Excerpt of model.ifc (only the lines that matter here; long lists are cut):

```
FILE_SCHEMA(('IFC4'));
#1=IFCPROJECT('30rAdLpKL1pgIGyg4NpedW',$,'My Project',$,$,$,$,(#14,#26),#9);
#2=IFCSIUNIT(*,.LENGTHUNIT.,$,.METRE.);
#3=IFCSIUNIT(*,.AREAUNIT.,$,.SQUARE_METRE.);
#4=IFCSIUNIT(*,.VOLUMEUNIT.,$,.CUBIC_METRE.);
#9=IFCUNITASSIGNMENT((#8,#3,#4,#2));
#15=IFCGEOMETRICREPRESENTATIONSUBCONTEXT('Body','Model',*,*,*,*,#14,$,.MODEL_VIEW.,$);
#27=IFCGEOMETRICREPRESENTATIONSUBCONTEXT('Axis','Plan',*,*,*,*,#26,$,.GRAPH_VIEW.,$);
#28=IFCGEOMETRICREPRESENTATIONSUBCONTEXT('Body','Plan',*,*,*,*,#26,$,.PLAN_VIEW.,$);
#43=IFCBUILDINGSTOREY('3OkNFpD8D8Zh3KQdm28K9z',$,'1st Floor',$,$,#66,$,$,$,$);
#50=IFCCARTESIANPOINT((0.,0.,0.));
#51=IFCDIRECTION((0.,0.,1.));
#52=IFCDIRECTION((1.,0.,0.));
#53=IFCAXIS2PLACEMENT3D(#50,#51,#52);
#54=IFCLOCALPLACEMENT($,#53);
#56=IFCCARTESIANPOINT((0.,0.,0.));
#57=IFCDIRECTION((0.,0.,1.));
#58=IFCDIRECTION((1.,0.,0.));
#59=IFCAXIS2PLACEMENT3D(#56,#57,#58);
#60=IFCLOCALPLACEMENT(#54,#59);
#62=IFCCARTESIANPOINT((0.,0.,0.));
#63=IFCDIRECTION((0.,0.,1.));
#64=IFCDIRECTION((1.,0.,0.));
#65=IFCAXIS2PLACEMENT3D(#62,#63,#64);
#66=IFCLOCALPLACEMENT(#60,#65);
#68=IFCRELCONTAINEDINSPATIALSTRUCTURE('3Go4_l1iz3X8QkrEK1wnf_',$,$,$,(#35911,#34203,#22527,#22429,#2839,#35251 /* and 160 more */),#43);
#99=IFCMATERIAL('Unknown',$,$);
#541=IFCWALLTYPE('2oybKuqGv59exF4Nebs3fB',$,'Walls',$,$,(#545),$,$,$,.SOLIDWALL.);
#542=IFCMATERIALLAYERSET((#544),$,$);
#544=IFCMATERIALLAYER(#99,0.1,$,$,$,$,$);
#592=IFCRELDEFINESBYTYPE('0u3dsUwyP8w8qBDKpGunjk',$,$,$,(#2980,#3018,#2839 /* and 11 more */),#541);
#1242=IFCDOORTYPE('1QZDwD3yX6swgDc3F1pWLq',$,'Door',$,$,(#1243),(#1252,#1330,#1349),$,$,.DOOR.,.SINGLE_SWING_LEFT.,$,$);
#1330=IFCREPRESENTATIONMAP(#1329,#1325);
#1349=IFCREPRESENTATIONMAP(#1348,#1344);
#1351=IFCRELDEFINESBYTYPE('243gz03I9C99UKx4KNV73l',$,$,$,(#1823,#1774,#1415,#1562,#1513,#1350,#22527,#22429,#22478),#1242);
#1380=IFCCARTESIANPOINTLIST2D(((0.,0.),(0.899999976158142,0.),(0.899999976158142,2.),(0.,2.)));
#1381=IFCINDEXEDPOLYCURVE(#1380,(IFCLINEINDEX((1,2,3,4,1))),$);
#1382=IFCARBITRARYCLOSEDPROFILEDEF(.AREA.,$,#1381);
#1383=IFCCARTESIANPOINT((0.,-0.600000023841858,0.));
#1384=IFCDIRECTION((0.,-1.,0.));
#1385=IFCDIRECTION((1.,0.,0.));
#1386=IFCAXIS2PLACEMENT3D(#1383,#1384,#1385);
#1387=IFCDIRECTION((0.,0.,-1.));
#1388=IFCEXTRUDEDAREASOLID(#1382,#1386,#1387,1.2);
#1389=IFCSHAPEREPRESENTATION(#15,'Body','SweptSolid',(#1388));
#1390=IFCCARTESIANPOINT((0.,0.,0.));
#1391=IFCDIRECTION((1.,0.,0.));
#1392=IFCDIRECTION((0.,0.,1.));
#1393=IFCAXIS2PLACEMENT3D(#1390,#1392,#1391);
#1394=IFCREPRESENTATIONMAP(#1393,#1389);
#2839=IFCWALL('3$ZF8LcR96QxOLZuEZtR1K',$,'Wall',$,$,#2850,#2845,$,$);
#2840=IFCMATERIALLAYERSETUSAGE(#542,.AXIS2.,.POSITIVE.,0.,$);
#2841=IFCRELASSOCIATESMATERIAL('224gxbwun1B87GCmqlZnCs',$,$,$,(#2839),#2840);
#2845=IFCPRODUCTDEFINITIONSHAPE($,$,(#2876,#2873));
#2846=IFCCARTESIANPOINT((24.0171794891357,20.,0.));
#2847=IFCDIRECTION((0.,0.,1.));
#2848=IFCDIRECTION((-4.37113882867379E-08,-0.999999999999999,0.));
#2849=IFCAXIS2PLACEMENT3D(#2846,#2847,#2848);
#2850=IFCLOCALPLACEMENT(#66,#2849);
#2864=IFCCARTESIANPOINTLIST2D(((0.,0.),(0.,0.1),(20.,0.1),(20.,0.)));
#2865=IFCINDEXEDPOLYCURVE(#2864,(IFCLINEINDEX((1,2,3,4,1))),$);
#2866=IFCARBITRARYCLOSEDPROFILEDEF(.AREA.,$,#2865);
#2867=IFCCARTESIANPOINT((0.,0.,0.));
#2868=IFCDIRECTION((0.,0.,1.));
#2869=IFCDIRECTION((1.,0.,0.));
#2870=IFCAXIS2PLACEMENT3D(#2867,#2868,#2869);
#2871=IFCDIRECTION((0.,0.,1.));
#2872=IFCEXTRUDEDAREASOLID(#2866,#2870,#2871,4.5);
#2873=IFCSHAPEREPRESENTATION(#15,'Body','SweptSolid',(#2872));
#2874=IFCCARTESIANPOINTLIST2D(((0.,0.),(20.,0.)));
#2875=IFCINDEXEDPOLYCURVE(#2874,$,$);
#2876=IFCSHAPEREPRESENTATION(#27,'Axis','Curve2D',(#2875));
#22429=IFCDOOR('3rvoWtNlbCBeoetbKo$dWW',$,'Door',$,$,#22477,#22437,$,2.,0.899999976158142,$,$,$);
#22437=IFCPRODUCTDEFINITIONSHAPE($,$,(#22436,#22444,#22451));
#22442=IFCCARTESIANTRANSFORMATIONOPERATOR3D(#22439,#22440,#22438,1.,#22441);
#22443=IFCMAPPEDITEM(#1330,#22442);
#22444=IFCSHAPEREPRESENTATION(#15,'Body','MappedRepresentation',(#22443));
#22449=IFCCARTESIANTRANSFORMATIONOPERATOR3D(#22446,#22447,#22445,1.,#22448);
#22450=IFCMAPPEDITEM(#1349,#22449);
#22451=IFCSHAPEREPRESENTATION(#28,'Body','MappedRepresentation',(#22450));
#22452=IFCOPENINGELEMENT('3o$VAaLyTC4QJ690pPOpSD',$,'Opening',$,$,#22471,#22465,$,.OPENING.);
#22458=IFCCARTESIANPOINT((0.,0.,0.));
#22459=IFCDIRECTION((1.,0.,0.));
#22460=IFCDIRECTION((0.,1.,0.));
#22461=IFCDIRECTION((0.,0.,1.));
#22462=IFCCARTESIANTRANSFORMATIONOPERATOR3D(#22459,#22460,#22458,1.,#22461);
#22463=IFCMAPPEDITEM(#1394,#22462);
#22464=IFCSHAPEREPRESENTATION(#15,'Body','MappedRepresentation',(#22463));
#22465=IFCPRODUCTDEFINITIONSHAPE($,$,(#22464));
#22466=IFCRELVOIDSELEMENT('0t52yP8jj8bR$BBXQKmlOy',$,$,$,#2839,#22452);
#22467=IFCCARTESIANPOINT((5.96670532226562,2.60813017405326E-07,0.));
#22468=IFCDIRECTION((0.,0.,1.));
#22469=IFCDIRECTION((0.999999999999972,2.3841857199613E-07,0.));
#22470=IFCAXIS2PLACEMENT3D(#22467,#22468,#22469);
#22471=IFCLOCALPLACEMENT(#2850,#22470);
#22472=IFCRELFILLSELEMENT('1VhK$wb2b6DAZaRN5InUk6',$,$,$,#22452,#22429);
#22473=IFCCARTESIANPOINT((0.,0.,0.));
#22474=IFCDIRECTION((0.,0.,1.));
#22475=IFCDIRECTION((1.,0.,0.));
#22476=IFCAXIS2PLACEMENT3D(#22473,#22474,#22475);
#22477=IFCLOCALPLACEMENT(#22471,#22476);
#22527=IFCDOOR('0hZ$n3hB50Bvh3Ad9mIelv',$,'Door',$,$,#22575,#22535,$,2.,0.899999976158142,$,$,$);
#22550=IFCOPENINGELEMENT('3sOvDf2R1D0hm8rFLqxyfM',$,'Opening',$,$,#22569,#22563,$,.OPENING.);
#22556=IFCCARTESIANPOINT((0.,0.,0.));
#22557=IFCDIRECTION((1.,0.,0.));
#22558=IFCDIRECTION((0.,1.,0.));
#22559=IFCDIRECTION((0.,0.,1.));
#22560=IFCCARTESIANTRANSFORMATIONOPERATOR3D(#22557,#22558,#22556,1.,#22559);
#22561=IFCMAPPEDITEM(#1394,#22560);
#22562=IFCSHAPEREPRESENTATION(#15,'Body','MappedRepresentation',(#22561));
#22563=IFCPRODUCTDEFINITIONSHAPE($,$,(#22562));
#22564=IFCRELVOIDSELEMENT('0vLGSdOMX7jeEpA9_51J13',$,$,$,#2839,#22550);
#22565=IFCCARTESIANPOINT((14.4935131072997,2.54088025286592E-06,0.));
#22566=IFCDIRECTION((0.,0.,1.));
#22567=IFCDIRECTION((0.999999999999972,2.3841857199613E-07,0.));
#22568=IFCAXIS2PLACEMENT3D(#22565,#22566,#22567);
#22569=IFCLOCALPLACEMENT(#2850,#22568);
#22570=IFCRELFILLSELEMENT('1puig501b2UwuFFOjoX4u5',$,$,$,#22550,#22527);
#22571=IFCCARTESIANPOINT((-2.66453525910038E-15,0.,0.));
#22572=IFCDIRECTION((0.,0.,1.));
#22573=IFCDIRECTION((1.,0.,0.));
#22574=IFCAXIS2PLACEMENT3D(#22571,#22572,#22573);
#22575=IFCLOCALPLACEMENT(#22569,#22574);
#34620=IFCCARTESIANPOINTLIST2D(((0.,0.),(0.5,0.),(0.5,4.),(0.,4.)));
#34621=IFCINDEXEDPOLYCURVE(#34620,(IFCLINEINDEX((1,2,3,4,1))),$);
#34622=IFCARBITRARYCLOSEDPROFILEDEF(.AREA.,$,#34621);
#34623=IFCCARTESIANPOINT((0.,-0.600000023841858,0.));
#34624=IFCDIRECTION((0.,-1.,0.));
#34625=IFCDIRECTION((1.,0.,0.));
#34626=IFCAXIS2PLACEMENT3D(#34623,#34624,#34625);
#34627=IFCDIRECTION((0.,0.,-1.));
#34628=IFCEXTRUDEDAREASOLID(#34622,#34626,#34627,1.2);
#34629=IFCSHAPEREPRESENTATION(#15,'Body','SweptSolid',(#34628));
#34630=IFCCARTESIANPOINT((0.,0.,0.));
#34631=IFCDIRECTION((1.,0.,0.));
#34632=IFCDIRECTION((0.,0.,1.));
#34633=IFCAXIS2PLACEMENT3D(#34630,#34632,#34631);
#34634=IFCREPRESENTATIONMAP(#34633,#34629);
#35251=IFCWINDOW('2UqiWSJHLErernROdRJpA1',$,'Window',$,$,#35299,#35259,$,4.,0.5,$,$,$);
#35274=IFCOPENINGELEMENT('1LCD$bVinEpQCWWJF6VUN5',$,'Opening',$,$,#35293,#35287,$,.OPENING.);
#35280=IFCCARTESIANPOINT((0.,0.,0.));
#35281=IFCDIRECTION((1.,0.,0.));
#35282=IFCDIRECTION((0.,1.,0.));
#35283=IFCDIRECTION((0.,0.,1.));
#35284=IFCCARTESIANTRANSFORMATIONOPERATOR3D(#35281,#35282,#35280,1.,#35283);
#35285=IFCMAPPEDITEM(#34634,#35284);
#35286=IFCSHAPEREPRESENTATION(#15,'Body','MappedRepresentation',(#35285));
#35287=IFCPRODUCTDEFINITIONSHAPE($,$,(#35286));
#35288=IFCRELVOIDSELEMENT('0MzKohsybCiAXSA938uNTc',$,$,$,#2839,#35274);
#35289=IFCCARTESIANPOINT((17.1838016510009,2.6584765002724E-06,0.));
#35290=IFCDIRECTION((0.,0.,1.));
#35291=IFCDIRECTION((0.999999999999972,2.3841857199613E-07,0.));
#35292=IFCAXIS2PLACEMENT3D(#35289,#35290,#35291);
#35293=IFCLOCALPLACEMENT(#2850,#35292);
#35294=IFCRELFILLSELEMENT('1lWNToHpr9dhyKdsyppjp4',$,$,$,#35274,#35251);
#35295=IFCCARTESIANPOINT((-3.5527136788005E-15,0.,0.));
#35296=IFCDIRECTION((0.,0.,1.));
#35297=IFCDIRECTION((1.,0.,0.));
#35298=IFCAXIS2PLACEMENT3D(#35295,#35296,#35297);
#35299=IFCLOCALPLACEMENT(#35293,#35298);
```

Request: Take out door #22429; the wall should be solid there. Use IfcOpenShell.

```python
import ifcopenshell
import ifcopenshell.api.feature
import ifcopenshell.api.root
import ifcopenshell.geom
import ifcopenshell.util.shape

model = ifcopenshell.open("model.ifc")
settings = ifcopenshell.geom.settings()


def volume(element):
    """Net volume in cubic metres, openings subtracted."""
    shape = ifcopenshell.geom.create_shape(settings, element)
    return ifcopenshell.util.shape.get_volume(shape.geometry)


door = model.by_guid("3rvoWtNlbCBeoetbKo$dWW")
opening = door.FillsVoids[0].RelatingOpeningElement
wall = opening.VoidsElements[0].RelatingBuildingElement
before = volume(wall)

ifcopenshell.api.root.remove_product(model, product=door)
ifcopenshell.api.feature.remove_feature(model, feature=opening)

after = volume(wall)

print(f"wall volume {before:.3f} -> {after:.3f} m3")

model.write("model-out.ifc")
```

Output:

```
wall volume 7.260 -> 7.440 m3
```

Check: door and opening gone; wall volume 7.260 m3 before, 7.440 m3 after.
